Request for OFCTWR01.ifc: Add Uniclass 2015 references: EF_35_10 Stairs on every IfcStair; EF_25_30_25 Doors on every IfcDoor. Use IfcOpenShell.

First a look at what the model holds.

```python
import ifcopenshell

model = ifcopenshell.open("OFCTWR01.ifc")
print(model.schema)
print("classifications:", [c.Name for c in model.by_type("IfcClassification")])
for ifc_class in ("IfcDoor", "IfcRoof", "IfcStair", "IfcWall", "IfcWindow"):
    print(ifc_class, len(model.by_type(ifc_class)))
```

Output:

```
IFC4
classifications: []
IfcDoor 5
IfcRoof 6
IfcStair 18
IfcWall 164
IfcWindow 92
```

```python
import ifcopenshell
import ifcopenshell.api.classification

model = ifcopenshell.open("OFCTWR01.ifc")

system = ifcopenshell.api.classification.add_classification(model, classification="Uniclass 2015")

codes = {
    "IfcStair": ("EF_35_10", "Stairs"),
    "IfcDoor": ("EF_25_30_25", "Doors"),
}
for ifc_class, (code, name) in codes.items():
    products = model.by_type(ifc_class)
    ifcopenshell.api.classification.add_reference(
        model, products=products, classification=system, identification=code, name=name
    )
    print(code, len(products))

model.write("OFCTWR01_rev.ifc")
```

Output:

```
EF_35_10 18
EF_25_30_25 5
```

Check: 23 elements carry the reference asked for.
